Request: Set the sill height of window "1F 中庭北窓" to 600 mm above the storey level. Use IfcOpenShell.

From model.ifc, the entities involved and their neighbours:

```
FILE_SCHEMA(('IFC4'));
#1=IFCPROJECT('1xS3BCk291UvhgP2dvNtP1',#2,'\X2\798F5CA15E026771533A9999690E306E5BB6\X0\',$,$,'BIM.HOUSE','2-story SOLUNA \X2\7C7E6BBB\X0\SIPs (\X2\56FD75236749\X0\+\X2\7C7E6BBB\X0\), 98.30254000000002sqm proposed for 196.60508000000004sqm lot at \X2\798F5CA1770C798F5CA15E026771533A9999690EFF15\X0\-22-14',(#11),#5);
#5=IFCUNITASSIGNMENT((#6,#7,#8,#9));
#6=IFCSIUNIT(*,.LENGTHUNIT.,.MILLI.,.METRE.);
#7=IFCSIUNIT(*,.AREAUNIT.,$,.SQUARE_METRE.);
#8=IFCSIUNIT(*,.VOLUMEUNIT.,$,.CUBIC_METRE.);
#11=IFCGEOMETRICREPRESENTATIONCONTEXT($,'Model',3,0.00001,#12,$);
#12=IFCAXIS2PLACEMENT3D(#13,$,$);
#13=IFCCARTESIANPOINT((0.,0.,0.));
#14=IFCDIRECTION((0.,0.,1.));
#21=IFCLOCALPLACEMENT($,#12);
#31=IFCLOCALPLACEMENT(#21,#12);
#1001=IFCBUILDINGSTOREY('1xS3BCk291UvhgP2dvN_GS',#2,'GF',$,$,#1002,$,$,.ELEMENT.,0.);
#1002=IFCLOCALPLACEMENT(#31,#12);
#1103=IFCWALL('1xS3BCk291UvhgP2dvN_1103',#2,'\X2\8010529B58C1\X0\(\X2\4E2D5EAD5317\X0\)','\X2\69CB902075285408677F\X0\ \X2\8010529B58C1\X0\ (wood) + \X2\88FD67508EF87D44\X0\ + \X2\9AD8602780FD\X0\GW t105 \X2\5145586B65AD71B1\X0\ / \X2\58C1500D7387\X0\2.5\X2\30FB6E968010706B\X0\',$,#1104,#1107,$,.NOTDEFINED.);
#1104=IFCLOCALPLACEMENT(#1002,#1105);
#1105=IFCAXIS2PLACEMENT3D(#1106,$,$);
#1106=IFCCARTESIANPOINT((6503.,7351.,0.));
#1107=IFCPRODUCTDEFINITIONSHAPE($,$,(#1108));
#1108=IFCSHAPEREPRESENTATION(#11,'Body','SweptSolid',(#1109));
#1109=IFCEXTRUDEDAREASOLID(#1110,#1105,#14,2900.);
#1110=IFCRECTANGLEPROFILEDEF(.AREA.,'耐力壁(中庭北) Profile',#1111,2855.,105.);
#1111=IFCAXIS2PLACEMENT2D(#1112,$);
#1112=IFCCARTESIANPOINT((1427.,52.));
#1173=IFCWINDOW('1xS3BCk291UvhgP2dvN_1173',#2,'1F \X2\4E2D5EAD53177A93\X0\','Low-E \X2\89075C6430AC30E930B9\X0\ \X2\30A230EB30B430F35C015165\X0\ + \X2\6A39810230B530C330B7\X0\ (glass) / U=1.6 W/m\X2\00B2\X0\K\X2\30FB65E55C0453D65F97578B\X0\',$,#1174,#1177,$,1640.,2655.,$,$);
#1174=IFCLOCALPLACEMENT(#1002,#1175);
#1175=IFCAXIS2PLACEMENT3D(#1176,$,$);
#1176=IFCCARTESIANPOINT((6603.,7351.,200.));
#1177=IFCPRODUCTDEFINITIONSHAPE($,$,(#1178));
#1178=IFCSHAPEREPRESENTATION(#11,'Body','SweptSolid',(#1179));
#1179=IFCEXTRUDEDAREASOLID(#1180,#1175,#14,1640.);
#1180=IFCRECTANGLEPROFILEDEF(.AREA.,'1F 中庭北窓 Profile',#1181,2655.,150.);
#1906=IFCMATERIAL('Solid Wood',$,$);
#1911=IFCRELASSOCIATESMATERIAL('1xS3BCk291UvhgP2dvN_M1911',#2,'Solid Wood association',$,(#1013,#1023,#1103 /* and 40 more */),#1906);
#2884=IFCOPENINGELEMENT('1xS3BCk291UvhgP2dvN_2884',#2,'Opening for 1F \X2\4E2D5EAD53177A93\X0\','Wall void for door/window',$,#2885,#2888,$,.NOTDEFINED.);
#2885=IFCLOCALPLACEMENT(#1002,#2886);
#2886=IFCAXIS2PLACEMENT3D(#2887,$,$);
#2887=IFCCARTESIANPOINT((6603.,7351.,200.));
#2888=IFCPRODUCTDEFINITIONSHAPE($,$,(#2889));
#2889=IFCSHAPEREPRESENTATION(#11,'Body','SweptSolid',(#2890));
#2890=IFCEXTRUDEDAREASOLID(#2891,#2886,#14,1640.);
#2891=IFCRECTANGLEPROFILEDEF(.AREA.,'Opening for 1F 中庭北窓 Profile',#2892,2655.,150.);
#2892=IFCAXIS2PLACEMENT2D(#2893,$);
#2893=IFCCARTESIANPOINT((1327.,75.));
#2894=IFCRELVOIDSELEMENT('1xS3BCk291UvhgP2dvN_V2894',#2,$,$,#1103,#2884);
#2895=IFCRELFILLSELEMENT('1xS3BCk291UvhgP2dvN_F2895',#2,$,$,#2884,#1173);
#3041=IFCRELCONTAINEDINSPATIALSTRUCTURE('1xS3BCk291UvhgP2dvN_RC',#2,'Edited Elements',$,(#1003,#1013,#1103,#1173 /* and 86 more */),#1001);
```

```python
import numpy as np
import ifcopenshell
import ifcopenshell.api.geometry
import ifcopenshell.geom
import ifcopenshell.util.element
import ifcopenshell.util.placement
import ifcopenshell.util.shape
import ifcopenshell.util.unit

model = ifcopenshell.open("model.ifc")
unit_scale = ifcopenshell.util.unit.calculate_unit_scale(model)

window = model.by_guid("1xS3BCk291UvhgP2dvN_1173")
opening = window.FillsVoids[0].RelatingOpeningElement
storey = ifcopenshell.util.element.get_container(window, ifc_class="IfcBuildingStorey")
level = ifcopenshell.util.placement.get_local_placement(storey.ObjectPlacement)[2, 3]

# The opening's origin need not be at the sill, so measure its lowest point.
shape = ifcopenshell.geom.create_shape(ifcopenshell.geom.settings(), opening)
bottom = ifcopenshell.util.shape.get_shape_bottom_elevation(shape, shape.geometry) / unit_scale
dz = level + 600.0 - bottom

shift = np.array([0.0, 0.0, dz])
# The window is not placed relative to its opening, so move both.
for product in (opening, window):
    matrix = ifcopenshell.util.placement.get_local_placement(product.ObjectPlacement)
    matrix[:3, 3] += shift
    ifcopenshell.api.geometry.edit_object_placement(model, product=product, matrix=matrix, is_si=False)

print(f"moved by {dz * unit_scale:+.3f} m")

model.write("model_rev.ifc")
```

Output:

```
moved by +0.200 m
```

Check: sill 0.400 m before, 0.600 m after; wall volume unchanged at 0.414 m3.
